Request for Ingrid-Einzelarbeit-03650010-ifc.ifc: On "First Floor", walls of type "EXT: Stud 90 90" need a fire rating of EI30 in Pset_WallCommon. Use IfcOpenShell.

First a look at what the model holds.

```python
import ifcopenshell
import ifcopenshell.util.element

model = ifcopenshell.open("Ingrid-Einzelarbeit-03650010-ifc.ifc")
print(model.schema)
storey = next(s for s in model.by_type("IfcBuildingStorey") if s.Name == "First Floor")
walls = [e for e in ifcopenshell.util.element.get_decomposition(storey) if e.is_a("IfcWall")]
seen = {}
for e in walls:
    element_type = ifcopenshell.util.element.get_type(e)
    key = (element_type.Name if element_type != e and element_type else None, ifcopenshell.util.element.get_pset(e, "Pset_WallCommon", "FireRating"))
    seen[key] = seen.get(key, 0) + 1
for (name, value), count in sorted(seen.items(), key=str):
    print(count, "x", name, "|", value)
```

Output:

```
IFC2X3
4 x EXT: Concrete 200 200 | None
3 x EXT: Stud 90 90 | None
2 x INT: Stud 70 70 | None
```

```python
import ifcopenshell
import ifcopenshell.api.pset
import ifcopenshell.util.element

model = ifcopenshell.open("Ingrid-Einzelarbeit-03650010-ifc.ifc")

storey = next(s for s in model.by_type("IfcBuildingStorey") if s.Name == "First Floor")
walls = [e for e in ifcopenshell.util.element.get_decomposition(storey) if e.is_a("IfcWall")]

count = 0
for e in walls:
    element_type = ifcopenshell.util.element.get_type(e)
    if element_type in (None, e) or element_type.Name != "EXT: Stud 90 90":
        continue
    # add_pset returns the element's existing set when there is one.
    pset = ifcopenshell.api.pset.add_pset(model, product=e, name="Pset_WallCommon")
    ifcopenshell.api.pset.edit_pset(model, pset=pset, properties={"FireRating": "EI30"})
    count += 1

print(count, "walls updated")

model.write("Ingrid-Einzelarbeit-03650010-ifc-out.ifc")
```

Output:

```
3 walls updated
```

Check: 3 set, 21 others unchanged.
